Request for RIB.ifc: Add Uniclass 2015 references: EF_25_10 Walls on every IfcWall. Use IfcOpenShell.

First a look at what the model holds.

```python
import ifcopenshell

model = ifcopenshell.open("RIB.ifc")
print(model.schema)
print("classifications:", [c.Name for c in model.by_type("IfcClassification")])
for ifc_class in ("IfcDoor", "IfcRoof", "IfcStair", "IfcWall", "IfcWindow"):
    print(ifc_class, len(model.by_type(ifc_class)))
```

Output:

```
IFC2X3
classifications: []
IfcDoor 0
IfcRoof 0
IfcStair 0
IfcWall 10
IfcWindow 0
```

```python
import ifcopenshell
import ifcopenshell.api.classification

model = ifcopenshell.open("RIB.ifc")

# IFC2X3 requires Source and Edition and has no link from the project to the system.
system = model.create_entity("IfcClassification", Source="NBS", Edition="2015", Name="Uniclass 2015")

codes = {
    "IfcWall": ("EF_25_10", "Walls"),
}
for ifc_class, (code, name) in codes.items():
    products = model.by_type(ifc_class)
    ifcopenshell.api.classification.add_reference(
        model, products=products, classification=system, identification=code, name=name
    )
    print(code, len(products))

model.write("RIB_rev.ifc")
```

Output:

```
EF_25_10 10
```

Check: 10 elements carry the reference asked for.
